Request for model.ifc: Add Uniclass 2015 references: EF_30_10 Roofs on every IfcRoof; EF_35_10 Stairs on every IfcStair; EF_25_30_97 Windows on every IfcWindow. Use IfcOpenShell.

First a look at what the model holds.

```python
import ifcopenshell

model = ifcopenshell.open("model.ifc")
print(model.schema)
print("classifications:", [c.Name for c in model.by_type("IfcClassification")])
for ifc_class in ("IfcDoor", "IfcRoof", "IfcStair", "IfcWall", "IfcWindow"):
    print(ifc_class, len(model.by_type(ifc_class)))
```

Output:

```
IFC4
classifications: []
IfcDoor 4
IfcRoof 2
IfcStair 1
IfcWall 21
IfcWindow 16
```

```python
import ifcopenshell
import ifcopenshell.api.classification

model = ifcopenshell.open("model.ifc")

system = ifcopenshell.api.classification.add_classification(model, classification="Uniclass 2015")

codes = {
    "IfcRoof": ("EF_30_10", "Roofs"),
    "IfcStair": ("EF_35_10", "Stairs"),
    "IfcWindow": ("EF_25_30_97", "Windows"),
}
for ifc_class, (code, name) in codes.items():
    products = model.by_type(ifc_class)
    ifcopenshell.api.classification.add_reference(
        model, products=products, classification=system, identification=code, name=name
    )
    print(code, len(products))

model.write("model_updated.ifc")
```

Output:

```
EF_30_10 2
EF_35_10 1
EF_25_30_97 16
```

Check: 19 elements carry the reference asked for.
